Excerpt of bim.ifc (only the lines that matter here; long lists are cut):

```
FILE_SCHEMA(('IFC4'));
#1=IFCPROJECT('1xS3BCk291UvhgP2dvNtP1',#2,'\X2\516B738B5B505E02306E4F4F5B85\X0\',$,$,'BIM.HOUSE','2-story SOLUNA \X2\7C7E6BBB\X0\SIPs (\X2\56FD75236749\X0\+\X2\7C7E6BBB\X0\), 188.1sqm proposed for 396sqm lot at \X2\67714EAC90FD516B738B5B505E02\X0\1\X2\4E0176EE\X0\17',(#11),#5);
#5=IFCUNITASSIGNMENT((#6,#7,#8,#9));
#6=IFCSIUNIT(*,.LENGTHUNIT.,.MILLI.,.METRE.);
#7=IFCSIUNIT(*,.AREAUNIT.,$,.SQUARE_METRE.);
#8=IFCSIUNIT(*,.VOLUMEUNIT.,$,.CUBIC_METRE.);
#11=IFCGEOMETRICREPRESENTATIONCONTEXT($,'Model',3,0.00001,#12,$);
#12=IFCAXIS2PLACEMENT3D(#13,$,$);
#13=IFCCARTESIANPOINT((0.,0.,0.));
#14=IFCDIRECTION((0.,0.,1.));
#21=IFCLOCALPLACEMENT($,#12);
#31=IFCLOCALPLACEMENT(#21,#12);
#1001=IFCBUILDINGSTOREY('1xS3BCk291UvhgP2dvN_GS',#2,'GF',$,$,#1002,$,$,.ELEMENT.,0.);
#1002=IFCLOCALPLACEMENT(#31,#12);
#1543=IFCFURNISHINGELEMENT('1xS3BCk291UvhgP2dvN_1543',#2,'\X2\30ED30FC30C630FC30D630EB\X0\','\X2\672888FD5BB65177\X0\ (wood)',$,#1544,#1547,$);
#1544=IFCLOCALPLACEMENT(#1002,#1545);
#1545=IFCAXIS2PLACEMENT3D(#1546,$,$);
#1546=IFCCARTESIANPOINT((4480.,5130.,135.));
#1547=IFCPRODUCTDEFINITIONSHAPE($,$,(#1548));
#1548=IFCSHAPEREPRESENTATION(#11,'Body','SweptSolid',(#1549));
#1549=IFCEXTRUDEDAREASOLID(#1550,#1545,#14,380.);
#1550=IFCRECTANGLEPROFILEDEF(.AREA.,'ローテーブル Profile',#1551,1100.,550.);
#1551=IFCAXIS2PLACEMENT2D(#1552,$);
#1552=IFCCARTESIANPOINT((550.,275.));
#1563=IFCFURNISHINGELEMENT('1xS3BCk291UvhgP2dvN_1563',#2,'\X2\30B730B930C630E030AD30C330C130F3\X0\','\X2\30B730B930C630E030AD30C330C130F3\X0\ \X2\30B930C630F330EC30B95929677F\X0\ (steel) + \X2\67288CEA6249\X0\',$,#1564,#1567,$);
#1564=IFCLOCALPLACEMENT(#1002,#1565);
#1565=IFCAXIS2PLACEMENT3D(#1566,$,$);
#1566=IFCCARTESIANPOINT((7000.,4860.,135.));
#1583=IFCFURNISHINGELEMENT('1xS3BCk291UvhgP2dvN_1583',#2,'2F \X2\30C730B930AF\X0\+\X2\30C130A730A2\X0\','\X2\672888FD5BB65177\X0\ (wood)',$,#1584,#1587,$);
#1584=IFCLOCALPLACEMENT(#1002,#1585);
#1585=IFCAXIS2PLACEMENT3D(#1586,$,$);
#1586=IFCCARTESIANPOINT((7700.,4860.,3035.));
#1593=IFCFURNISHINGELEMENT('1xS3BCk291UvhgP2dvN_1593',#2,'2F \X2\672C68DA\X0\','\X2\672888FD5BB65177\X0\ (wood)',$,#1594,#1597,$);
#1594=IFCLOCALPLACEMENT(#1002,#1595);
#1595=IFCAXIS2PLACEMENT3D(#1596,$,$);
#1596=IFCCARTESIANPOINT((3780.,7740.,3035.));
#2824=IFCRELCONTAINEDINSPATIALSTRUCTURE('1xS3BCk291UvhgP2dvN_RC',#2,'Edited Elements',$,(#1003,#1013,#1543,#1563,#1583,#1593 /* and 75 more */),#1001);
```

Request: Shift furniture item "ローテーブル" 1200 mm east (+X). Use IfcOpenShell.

```python
import ifcopenshell
import ifcopenshell.api.geometry
import ifcopenshell.util.placement
import ifcopenshell.util.unit

model = ifcopenshell.open("bim.ifc")
unit_scale = ifcopenshell.util.unit.calculate_unit_scale(model)

item = model.by_guid("1xS3BCk291UvhgP2dvN_1543")
matrix = ifcopenshell.util.placement.get_local_placement(item.ObjectPlacement)
matrix[0, 3] += 1.2 / unit_scale
ifcopenshell.api.geometry.edit_object_placement(model, product=item, matrix=matrix, is_si=False)

print(ifcopenshell.util.placement.get_local_placement(item.ObjectPlacement).round(3) + 0.0)

model.write("bim_rev.ifc")
```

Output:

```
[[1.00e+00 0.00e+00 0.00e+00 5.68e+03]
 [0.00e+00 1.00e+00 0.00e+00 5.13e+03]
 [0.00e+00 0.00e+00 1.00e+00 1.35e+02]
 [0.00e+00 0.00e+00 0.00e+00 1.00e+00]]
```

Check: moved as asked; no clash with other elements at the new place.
